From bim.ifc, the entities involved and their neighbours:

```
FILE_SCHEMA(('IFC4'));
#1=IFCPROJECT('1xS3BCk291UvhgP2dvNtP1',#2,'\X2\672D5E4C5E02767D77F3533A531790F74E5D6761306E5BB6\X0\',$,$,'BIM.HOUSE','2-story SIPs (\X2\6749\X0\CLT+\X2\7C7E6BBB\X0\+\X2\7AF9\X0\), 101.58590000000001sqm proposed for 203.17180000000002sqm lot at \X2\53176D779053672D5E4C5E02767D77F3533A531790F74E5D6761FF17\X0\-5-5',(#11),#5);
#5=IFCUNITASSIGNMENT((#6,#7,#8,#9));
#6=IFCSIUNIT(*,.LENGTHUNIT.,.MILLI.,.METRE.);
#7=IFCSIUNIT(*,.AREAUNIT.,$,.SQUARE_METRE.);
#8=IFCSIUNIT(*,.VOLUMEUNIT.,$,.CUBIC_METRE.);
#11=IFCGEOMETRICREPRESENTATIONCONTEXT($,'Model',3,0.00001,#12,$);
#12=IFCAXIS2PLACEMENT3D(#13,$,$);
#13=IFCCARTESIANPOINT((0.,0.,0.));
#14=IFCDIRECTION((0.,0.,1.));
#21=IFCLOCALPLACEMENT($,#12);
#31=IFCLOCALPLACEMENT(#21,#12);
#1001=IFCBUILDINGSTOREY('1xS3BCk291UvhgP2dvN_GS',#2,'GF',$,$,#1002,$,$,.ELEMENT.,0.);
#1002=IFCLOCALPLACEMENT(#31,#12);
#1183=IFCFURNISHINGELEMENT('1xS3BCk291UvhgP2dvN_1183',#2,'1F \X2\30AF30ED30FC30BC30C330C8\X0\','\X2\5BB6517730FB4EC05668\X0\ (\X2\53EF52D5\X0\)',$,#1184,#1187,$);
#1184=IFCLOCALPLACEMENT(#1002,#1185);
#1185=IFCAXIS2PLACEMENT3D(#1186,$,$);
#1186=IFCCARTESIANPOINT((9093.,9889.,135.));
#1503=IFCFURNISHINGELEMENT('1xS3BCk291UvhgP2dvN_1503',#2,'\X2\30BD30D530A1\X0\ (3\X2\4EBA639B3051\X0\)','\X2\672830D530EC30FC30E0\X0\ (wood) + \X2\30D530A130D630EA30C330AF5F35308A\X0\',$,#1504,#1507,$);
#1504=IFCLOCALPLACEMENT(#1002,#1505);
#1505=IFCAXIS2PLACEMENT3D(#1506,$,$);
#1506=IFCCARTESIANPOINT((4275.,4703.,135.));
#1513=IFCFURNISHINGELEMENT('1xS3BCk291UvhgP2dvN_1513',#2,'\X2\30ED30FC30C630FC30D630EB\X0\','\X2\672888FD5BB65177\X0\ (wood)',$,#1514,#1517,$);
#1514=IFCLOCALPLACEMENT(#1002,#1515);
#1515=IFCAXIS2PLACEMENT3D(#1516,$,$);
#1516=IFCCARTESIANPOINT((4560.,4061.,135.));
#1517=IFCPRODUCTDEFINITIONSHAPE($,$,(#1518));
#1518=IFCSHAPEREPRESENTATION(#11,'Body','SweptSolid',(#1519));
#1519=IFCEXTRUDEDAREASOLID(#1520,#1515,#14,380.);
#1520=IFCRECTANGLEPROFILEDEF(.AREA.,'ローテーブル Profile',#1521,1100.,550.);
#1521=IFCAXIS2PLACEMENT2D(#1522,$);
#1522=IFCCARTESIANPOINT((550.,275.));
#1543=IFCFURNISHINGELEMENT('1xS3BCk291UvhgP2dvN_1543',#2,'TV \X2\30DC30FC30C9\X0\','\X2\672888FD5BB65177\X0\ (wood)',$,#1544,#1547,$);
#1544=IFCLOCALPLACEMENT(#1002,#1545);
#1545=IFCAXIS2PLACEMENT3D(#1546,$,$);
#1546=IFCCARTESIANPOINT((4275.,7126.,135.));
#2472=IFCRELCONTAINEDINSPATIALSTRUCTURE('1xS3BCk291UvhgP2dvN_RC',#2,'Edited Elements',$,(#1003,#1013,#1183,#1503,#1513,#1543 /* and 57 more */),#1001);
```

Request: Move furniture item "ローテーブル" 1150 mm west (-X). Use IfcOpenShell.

```python
import ifcopenshell
import ifcopenshell.api.geometry
import ifcopenshell.util.placement
import ifcopenshell.util.unit

model = ifcopenshell.open("bim.ifc")
unit_scale = ifcopenshell.util.unit.calculate_unit_scale(model)

item = model.by_id(1513)
matrix = ifcopenshell.util.placement.get_local_placement(item.ObjectPlacement)
matrix[0, 3] -= 1.15 / unit_scale
ifcopenshell.api.geometry.edit_object_placement(model, product=item, matrix=matrix, is_si=False)

print(ifcopenshell.util.placement.get_local_placement(item.ObjectPlacement).round(3) + 0.0)

model.write("bim_v2.ifc")
```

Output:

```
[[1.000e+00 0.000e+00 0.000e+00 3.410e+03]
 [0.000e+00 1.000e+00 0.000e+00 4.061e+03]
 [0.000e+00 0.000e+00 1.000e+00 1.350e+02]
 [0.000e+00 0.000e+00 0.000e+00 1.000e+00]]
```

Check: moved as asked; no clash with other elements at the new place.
